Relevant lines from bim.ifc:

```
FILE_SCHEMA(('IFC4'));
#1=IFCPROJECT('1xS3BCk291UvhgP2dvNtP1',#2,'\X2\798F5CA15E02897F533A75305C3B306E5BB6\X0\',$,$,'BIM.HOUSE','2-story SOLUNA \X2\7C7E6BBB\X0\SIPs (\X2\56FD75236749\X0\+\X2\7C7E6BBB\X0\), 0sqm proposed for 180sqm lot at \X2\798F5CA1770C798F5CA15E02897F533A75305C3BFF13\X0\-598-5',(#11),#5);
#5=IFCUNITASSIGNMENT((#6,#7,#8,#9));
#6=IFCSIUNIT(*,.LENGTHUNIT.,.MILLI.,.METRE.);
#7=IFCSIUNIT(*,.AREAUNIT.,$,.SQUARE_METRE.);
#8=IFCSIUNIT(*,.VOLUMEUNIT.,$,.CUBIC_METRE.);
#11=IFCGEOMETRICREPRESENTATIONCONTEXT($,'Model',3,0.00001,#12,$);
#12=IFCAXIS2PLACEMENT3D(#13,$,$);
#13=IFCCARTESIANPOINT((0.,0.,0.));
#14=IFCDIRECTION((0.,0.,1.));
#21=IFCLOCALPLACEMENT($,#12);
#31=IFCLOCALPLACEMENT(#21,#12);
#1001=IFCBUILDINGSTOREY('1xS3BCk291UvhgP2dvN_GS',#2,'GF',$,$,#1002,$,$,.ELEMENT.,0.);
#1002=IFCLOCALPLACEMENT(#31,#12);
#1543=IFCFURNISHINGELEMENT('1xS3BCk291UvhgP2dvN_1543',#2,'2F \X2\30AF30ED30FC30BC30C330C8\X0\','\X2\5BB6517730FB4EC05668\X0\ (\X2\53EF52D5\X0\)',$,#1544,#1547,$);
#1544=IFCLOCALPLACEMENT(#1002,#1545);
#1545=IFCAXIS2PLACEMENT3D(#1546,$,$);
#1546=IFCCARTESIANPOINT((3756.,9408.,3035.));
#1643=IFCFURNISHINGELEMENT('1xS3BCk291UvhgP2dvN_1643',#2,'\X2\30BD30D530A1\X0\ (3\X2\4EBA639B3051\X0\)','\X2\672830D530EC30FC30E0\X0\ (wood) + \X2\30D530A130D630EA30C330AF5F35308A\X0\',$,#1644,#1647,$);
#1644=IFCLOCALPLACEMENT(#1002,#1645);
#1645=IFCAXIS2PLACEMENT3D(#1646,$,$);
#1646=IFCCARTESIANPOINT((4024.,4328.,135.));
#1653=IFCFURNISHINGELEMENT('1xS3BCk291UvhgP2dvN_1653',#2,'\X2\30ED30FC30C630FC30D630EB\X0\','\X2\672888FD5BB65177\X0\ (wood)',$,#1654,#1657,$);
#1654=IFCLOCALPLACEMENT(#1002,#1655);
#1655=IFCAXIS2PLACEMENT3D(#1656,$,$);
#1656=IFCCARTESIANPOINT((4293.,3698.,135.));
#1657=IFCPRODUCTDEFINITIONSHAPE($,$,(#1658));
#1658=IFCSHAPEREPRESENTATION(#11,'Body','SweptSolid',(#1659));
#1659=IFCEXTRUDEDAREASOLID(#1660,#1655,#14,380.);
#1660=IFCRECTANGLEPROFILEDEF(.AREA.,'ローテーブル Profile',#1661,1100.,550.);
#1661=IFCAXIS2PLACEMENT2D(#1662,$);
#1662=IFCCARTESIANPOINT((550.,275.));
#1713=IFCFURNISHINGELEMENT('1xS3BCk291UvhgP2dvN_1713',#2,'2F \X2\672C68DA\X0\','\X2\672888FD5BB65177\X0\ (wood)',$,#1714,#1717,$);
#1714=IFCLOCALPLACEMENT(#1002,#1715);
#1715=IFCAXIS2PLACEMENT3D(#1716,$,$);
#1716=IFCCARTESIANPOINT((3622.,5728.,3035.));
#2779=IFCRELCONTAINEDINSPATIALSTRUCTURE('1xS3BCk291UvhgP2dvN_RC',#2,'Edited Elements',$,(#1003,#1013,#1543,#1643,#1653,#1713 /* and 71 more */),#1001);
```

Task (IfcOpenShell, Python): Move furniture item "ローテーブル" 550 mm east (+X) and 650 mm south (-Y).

```python
import ifcopenshell
import ifcopenshell.api.geometry
import ifcopenshell.util.placement

model = ifcopenshell.open("bim.ifc")

item = model.by_guid("1xS3BCk291UvhgP2dvN_1653")
matrix = ifcopenshell.util.placement.get_local_placement(item.ObjectPlacement)
matrix[0, 3] += 550.0
matrix[1, 3] -= 650.0
ifcopenshell.api.geometry.edit_object_placement(model, product=item, matrix=matrix, is_si=False)

print(ifcopenshell.util.placement.get_local_placement(item.ObjectPlacement).round(3) + 0.0)

model.write("bim_v2.ifc")
```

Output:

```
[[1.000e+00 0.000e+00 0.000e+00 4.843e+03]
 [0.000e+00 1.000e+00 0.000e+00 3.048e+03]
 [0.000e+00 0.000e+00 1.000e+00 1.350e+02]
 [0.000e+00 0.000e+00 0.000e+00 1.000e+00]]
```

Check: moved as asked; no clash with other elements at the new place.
